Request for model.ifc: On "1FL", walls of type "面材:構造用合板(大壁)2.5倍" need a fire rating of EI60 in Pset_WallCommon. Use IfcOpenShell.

First a look at what the model holds.

```python
import ifcopenshell
import ifcopenshell.util.element

model = ifcopenshell.open("model.ifc")
print(model.schema)
storey = next(s for s in model.by_type("IfcBuildingStorey") if s.Name == "1FL")
walls = [e for e in ifcopenshell.util.element.get_decomposition(storey) if e.is_a("IfcWall")]
seen = {}
for e in walls:
    element_type = ifcopenshell.util.element.get_type(e)
    key = (element_type.Name if element_type != e and element_type else None, ifcopenshell.util.element.get_pset(e, "Pset_WallCommon", "FireRating"))
    seen[key] = seen.get(key, 0) + 1
for (name, value), count in sorted(seen.items(), key=str):
    print(count, "x", name, "|", value)
```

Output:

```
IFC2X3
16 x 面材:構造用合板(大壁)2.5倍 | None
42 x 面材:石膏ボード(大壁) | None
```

```python
import ifcopenshell
import ifcopenshell.api.pset
import ifcopenshell.util.element

model = ifcopenshell.open("model.ifc")

storey = next(s for s in model.by_type("IfcBuildingStorey") if s.Name == "1FL")
walls = [e for e in ifcopenshell.util.element.get_decomposition(storey) if e.is_a("IfcWall")]

count = 0
for e in walls:
    element_type = ifcopenshell.util.element.get_type(e)
    if element_type in (None, e) or element_type.Name != "面材:構造用合板(大壁)2.5倍":
        continue
    # add_pset returns the element's existing set when there is one.
    pset = ifcopenshell.api.pset.add_pset(model, product=e, name="Pset_WallCommon")
    ifcopenshell.api.pset.edit_pset(model, pset=pset, properties={"FireRating": "EI60"})
    count += 1

print(count, "walls updated")

model.write("model_rev.ifc")
```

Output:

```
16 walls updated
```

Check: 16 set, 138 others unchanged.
